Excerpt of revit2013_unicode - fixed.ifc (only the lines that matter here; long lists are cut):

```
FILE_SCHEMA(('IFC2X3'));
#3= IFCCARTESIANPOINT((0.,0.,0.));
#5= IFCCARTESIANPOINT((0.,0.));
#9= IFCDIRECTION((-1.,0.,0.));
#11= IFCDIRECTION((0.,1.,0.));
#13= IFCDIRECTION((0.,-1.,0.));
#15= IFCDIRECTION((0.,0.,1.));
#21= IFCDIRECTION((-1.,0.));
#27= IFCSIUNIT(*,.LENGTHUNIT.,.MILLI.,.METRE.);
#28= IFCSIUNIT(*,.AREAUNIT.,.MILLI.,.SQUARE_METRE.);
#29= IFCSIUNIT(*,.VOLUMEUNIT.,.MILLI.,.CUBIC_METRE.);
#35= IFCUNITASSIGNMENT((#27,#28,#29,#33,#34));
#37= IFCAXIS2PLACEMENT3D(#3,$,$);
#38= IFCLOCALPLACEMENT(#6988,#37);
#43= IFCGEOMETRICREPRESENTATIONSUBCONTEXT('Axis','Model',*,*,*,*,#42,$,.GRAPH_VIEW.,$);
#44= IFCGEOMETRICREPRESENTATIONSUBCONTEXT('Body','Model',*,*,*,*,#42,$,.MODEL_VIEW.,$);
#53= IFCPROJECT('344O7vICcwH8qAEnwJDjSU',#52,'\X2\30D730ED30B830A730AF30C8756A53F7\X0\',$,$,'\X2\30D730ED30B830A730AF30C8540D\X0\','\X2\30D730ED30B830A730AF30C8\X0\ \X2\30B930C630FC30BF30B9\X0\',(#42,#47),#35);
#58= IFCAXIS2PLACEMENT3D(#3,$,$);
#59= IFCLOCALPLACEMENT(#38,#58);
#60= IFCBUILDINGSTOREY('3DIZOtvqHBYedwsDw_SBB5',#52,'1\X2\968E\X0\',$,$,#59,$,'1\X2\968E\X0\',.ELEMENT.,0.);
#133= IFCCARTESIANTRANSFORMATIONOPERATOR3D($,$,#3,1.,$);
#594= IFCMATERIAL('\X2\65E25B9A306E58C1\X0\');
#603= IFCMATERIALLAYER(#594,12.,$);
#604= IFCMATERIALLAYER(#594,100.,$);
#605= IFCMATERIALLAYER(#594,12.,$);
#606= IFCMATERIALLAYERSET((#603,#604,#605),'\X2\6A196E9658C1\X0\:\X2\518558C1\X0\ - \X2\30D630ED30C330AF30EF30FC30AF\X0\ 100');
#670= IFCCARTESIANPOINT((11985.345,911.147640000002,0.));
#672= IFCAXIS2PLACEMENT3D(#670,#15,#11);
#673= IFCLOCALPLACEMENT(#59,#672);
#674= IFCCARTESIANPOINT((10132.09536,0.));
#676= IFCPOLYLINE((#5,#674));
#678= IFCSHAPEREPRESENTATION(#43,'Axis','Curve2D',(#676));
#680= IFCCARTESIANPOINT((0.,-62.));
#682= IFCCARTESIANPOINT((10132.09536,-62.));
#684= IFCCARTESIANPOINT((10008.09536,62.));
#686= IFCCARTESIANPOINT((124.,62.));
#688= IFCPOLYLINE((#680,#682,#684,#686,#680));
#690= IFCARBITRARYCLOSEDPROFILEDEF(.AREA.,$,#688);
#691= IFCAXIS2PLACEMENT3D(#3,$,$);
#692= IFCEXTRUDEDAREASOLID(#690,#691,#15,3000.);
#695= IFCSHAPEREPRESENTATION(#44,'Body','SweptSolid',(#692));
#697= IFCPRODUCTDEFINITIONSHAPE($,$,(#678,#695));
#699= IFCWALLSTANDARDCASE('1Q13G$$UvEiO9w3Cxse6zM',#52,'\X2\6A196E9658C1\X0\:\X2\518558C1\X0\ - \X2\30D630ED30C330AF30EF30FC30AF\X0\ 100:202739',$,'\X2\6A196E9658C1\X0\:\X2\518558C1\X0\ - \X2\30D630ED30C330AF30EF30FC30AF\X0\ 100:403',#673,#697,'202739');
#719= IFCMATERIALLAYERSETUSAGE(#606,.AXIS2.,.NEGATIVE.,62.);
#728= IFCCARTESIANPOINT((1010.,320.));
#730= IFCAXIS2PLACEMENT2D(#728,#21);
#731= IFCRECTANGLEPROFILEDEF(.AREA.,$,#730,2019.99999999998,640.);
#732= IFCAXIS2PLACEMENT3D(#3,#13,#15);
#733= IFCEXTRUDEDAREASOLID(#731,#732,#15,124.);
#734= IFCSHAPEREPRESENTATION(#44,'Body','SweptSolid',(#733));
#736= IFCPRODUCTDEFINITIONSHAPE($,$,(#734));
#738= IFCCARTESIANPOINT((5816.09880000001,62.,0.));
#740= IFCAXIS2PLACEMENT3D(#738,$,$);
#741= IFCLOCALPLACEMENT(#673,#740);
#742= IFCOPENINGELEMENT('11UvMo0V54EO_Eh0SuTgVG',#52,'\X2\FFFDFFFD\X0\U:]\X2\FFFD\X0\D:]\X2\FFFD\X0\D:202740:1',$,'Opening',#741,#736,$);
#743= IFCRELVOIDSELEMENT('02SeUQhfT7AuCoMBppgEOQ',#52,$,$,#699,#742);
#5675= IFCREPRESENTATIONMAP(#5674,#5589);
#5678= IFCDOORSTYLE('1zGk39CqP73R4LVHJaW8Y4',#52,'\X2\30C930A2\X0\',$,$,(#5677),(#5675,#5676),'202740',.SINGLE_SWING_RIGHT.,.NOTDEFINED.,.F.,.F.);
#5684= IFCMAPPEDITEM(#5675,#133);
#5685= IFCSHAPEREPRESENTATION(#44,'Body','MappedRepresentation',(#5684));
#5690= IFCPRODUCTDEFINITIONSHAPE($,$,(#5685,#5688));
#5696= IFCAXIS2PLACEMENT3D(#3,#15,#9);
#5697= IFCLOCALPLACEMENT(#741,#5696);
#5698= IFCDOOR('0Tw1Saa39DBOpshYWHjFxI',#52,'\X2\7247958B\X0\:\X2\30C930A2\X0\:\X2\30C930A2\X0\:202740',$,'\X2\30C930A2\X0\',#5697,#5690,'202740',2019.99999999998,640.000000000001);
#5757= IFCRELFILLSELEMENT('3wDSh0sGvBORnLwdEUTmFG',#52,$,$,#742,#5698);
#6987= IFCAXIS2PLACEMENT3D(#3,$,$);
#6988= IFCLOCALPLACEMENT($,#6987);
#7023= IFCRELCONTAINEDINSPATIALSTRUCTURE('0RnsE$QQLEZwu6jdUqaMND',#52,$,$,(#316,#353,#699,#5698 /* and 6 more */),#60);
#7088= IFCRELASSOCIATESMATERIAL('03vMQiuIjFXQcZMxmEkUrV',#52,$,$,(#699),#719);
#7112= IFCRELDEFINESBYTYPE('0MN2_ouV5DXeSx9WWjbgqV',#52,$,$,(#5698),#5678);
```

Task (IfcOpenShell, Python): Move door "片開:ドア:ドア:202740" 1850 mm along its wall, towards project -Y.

```python
import ifcopenshell
import ifcopenshell.api.geometry
import ifcopenshell.util.placement

model = ifcopenshell.open("revit2013_unicode - fixed.ifc")

door = model.by_id(5698)
opening = door.FillsVoids[0].RelatingOpeningElement
wall = opening.VoidsElements[0].RelatingBuildingElement

wall_matrix = ifcopenshell.util.placement.get_local_placement(wall.ObjectPlacement)
shift = wall_matrix[:3, 0] * -1850.0
before = ifcopenshell.util.placement.get_local_placement(door.ObjectPlacement)[:3, 3].copy()

# The door is placed relative to its opening, so it follows when the opening moves.
matrix = ifcopenshell.util.placement.get_local_placement(opening.ObjectPlacement)
matrix[:3, 3] += shift
ifcopenshell.api.geometry.edit_object_placement(
    model, product=opening, matrix=matrix, is_si=False, should_transform_children=True
)

after = ifcopenshell.util.placement.get_local_placement(door.ObjectPlacement)[:3, 3]
print("door moved by", (after - before).round(3) + 0.0)

model.write("revit2013_unicode - fixed_rev.ifc")
```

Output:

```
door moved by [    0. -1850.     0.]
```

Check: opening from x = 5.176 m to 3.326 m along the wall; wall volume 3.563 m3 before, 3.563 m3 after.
